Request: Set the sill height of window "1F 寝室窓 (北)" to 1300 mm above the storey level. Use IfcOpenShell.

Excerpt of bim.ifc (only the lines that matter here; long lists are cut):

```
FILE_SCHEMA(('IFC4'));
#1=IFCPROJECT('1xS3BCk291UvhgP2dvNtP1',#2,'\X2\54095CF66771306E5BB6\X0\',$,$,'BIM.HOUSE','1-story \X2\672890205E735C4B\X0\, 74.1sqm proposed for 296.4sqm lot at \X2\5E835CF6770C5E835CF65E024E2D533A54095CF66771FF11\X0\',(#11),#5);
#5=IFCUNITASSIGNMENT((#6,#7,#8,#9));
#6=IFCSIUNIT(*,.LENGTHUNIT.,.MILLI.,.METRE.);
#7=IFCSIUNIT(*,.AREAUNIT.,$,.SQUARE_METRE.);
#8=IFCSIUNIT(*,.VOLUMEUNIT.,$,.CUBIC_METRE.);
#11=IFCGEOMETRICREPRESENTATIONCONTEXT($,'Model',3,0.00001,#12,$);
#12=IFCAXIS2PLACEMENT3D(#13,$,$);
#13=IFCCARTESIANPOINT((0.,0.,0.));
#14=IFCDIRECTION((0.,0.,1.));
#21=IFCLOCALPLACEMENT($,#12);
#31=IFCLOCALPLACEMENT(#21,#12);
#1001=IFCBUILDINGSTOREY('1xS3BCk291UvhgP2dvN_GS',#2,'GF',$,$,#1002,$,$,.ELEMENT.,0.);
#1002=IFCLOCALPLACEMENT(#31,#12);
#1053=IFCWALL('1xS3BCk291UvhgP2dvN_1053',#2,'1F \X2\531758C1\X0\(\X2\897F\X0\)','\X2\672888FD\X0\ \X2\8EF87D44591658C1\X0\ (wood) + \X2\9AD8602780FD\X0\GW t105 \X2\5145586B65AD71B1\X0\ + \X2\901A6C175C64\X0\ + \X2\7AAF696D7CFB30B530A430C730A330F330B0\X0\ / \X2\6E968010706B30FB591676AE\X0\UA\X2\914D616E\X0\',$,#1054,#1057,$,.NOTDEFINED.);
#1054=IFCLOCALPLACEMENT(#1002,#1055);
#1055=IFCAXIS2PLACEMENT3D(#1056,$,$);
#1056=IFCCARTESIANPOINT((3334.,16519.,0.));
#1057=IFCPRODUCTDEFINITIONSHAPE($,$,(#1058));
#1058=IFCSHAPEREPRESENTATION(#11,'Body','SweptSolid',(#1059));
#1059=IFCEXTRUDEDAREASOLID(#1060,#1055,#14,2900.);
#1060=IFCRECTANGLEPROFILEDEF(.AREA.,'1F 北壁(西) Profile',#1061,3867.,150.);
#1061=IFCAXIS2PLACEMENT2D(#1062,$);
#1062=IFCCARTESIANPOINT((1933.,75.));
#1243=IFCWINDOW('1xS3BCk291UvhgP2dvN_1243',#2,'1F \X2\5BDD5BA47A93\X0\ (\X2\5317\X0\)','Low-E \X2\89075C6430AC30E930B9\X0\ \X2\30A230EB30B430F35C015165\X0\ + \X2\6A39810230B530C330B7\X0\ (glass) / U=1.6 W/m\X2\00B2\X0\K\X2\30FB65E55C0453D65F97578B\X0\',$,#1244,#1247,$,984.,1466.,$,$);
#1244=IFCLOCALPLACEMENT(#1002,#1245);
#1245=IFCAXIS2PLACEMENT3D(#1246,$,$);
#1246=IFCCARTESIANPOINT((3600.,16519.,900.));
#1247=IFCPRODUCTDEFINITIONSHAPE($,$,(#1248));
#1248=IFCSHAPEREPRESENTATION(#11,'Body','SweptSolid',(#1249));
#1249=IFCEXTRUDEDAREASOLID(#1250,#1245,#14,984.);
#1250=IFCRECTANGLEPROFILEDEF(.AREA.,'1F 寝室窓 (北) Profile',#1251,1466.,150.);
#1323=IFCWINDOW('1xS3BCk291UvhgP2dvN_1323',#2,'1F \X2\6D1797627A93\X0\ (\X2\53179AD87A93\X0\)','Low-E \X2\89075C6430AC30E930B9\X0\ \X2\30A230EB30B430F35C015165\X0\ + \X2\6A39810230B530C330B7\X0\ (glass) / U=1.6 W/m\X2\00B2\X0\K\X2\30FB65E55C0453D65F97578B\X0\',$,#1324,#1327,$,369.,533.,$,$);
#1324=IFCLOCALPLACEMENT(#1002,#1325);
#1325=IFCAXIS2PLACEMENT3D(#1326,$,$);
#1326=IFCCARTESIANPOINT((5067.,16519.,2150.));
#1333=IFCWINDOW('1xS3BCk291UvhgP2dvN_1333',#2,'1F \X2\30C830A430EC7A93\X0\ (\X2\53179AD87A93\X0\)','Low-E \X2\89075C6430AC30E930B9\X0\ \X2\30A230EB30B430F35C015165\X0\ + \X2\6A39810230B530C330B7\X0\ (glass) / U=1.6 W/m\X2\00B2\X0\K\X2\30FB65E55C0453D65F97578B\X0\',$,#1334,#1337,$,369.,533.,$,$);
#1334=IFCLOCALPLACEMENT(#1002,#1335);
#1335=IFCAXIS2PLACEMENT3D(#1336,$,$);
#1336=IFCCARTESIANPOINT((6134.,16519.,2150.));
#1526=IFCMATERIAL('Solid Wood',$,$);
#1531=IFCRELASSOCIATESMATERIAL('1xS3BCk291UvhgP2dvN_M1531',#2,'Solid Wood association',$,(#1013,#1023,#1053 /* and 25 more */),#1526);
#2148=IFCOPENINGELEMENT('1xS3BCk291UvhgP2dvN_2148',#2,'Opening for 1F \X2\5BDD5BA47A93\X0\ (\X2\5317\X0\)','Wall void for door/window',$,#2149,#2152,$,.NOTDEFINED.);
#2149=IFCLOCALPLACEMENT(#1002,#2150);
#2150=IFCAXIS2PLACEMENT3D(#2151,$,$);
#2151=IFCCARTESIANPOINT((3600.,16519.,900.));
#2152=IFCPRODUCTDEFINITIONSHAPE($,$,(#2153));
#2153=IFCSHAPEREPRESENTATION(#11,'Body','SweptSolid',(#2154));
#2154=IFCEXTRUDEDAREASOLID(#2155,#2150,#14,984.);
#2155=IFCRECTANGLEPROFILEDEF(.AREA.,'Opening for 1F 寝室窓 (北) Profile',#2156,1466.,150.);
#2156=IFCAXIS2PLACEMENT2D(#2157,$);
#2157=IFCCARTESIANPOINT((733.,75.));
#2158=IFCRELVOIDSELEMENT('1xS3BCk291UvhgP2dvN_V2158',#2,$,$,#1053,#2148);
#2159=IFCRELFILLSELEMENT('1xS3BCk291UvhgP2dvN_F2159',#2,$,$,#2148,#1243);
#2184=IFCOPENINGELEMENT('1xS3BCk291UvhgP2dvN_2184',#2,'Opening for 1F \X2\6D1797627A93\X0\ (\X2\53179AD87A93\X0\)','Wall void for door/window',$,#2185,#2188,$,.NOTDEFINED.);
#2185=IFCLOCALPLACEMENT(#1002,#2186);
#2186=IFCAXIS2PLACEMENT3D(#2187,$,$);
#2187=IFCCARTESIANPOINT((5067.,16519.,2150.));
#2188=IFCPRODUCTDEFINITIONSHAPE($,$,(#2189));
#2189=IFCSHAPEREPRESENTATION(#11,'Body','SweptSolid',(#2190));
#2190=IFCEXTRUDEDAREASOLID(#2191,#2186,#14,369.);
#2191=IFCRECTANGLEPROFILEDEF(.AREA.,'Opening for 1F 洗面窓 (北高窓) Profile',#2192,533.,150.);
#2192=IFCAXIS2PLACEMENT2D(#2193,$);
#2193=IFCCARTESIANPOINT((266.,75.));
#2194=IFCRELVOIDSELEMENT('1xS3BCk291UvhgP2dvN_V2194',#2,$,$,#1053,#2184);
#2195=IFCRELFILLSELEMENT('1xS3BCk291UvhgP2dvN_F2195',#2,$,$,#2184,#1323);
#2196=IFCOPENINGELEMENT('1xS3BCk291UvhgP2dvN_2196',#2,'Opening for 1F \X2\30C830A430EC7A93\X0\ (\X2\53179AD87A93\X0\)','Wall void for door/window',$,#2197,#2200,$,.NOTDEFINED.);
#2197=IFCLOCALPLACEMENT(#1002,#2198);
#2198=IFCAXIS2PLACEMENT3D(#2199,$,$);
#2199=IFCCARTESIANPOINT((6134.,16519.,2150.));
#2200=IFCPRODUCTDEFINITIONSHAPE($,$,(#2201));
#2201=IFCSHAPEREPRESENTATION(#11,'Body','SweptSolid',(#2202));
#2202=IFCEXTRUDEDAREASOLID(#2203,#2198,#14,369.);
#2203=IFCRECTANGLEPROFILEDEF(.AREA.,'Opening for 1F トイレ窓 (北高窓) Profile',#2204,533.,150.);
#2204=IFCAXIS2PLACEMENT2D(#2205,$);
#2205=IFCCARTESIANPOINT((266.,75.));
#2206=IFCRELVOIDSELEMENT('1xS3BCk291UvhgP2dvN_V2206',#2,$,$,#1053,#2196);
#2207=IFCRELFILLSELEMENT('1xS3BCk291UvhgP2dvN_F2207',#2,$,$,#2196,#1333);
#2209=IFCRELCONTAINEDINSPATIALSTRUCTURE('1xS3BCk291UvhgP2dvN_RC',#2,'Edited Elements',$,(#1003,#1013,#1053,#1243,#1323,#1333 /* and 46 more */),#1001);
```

```python
import numpy as np
import ifcopenshell
import ifcopenshell.api.geometry
import ifcopenshell.geom
import ifcopenshell.util.element
import ifcopenshell.util.placement
import ifcopenshell.util.shape
import ifcopenshell.util.unit

model = ifcopenshell.open("bim.ifc")
unit_scale = ifcopenshell.util.unit.calculate_unit_scale(model)

window = model.by_guid("1xS3BCk291UvhgP2dvN_1243")
opening = window.FillsVoids[0].RelatingOpeningElement
storey = ifcopenshell.util.element.get_container(window, ifc_class="IfcBuildingStorey")
level = ifcopenshell.util.placement.get_local_placement(storey.ObjectPlacement)[2, 3]

# The opening's origin need not be at the sill, so measure its lowest point.
shape = ifcopenshell.geom.create_shape(ifcopenshell.geom.settings(), opening)
bottom = ifcopenshell.util.shape.get_shape_bottom_elevation(shape, shape.geometry) / unit_scale
dz = level + 1.3 / unit_scale - bottom

shift = np.array([0.0, 0.0, dz])
# The window is not placed relative to its opening, so move both.
for product in (opening, window):
    matrix = ifcopenshell.util.placement.get_local_placement(product.ObjectPlacement)
    matrix[:3, 3] += shift
    ifcopenshell.api.geometry.edit_object_placement(model, product=product, matrix=matrix, is_si=False)

print(f"moved by {dz * unit_scale:+.3f} m")

model.write("bim_updated.ifc")
```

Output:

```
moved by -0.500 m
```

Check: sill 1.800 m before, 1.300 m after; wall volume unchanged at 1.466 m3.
